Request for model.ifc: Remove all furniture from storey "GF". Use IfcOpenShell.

First a look at what the model holds.

```python
import ifcopenshell
import ifcopenshell.util.element

model = ifcopenshell.open("model.ifc")
print(model.schema)
storey = next(s for s in model.by_type("IfcBuildingStorey") if s.Name == "GF")
furniture = [e for e in ifcopenshell.util.element.get_decomposition(storey) if e.is_a("IfcFurnishingElement")]
seen = {}
for e in furniture:
    element_type = ifcopenshell.util.element.get_type(e)
    name = element_type.Name if element_type not in (None, e) else None
    seen[name] = seen.get(name, 0) + 1
for name, count in sorted(seen.items(), key=str):
    print(count, "x", name)
```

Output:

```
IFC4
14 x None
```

```python
import ifcopenshell
import ifcopenshell.api.root
import ifcopenshell.util.element

model = ifcopenshell.open("model.ifc")

storey = next(s for s in model.by_type("IfcBuildingStorey") if s.Name == "GF")
furniture = [e for e in ifcopenshell.util.element.get_decomposition(storey) if e.is_a("IfcFurnishingElement")]

for e in furniture:
    ifcopenshell.api.root.remove_product(model, product=e)
print(len(furniture), "removed")

model.write("model-out.ifc")
```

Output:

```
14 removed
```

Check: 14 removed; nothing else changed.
